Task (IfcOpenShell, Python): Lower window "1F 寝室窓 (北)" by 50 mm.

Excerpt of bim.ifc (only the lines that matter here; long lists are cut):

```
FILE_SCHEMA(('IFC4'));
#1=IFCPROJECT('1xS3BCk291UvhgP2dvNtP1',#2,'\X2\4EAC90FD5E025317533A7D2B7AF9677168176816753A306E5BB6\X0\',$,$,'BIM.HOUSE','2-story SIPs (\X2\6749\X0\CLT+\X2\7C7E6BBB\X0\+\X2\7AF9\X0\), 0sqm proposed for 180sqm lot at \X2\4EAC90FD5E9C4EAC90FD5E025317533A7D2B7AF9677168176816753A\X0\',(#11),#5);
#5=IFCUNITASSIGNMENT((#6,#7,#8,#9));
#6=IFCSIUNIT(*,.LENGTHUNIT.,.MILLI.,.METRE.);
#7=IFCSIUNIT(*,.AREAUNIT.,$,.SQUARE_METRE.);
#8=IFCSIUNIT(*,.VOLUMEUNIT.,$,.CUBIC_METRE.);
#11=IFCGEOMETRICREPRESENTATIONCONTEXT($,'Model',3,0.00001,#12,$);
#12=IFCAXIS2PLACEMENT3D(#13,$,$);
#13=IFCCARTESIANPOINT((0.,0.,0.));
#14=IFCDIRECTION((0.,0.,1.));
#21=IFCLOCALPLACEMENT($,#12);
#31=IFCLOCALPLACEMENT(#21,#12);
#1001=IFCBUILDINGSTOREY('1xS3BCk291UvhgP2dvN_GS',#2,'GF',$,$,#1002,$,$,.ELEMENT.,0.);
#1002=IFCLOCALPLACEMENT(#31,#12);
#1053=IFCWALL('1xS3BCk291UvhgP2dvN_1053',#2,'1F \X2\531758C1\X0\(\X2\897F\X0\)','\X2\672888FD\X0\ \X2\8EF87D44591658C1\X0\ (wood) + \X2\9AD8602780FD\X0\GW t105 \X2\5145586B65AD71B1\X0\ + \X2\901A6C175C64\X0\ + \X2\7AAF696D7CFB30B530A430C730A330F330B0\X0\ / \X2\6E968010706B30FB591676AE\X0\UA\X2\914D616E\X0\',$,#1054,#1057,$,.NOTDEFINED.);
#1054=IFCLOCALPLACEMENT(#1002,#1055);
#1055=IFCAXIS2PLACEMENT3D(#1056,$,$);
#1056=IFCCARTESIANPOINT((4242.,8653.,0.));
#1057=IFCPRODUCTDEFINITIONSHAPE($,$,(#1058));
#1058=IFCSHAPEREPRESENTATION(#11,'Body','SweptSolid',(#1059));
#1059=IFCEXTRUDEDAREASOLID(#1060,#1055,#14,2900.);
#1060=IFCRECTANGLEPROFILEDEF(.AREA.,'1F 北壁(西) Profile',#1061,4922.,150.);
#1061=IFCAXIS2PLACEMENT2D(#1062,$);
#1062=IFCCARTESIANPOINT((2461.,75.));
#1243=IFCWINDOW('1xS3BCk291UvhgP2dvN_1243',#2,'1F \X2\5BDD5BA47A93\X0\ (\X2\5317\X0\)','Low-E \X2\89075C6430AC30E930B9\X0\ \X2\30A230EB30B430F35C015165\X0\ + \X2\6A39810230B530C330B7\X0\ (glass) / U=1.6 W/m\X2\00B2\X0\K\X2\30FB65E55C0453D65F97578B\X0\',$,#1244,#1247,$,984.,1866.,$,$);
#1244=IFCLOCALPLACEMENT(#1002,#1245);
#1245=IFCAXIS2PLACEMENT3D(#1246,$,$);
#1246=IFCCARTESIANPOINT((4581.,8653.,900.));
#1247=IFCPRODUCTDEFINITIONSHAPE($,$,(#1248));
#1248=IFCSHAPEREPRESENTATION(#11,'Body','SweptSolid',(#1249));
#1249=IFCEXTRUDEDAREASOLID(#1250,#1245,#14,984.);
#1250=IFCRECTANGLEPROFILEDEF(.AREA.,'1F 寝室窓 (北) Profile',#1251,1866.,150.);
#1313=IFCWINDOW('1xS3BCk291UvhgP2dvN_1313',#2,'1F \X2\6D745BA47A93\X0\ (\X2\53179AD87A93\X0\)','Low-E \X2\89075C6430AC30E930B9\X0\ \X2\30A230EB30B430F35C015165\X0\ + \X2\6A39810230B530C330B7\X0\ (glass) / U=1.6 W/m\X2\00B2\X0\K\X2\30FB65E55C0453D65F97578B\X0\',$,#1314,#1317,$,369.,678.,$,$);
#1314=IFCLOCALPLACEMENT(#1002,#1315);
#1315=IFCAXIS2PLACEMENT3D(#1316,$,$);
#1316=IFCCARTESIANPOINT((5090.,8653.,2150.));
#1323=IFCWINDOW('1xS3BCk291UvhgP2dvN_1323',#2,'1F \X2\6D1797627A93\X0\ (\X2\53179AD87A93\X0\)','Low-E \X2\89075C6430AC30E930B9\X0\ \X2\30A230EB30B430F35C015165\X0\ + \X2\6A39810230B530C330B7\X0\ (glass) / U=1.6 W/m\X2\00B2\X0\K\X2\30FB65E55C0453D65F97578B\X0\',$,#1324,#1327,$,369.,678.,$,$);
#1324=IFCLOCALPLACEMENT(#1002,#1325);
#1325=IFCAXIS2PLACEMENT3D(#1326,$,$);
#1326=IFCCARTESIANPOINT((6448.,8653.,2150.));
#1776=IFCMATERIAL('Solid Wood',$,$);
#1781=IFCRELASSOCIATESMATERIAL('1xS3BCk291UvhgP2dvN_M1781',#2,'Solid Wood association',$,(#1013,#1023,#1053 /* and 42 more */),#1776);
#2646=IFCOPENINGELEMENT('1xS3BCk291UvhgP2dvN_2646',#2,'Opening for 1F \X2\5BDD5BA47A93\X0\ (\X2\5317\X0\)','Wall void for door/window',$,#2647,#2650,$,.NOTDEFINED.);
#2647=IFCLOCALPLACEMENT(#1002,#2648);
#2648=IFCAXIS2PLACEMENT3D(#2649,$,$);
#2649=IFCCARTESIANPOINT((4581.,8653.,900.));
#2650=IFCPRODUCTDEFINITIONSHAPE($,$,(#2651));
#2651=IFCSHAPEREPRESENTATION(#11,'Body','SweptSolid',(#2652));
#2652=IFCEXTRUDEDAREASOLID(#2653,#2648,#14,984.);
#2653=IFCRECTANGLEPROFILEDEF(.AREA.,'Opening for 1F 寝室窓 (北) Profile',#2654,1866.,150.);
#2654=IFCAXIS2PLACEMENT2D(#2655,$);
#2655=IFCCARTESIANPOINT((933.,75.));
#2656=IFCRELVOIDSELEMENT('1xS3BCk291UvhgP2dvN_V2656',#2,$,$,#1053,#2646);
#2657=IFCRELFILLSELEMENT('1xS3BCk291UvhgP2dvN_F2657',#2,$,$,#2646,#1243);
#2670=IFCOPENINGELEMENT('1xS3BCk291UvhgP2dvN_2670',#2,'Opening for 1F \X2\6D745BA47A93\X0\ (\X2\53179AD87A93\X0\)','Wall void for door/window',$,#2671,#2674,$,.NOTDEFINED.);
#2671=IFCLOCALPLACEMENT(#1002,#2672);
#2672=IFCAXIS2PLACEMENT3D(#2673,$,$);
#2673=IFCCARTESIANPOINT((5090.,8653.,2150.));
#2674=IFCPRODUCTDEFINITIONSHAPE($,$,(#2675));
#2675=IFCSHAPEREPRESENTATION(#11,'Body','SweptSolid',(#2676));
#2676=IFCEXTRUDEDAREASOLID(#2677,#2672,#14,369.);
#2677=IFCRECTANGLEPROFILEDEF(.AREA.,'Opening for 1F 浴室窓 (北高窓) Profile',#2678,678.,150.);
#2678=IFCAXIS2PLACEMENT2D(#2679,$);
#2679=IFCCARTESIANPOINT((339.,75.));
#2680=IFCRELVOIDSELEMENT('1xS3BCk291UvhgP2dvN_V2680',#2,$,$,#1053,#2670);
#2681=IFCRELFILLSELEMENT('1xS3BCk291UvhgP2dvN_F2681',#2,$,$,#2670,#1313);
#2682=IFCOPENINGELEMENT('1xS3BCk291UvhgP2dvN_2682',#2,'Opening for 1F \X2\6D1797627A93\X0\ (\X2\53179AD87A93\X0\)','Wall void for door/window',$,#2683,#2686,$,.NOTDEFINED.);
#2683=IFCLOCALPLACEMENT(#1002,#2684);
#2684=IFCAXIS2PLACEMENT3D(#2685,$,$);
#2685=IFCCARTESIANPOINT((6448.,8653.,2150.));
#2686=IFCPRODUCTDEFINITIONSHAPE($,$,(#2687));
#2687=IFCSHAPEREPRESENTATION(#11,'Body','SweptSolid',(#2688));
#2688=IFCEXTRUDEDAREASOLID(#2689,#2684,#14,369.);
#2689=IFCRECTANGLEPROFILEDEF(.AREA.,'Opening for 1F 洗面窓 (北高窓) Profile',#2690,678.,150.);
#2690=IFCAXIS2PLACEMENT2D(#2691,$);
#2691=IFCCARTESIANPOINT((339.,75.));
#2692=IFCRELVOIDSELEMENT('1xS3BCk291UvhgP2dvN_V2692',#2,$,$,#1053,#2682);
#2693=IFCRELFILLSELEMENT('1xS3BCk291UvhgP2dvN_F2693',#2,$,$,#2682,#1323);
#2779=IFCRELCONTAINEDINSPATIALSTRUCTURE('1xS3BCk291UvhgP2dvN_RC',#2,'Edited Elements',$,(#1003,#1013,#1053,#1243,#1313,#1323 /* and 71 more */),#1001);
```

```python
import numpy as np
import ifcopenshell
import ifcopenshell.api.geometry
import ifcopenshell.util.placement
import ifcopenshell.util.unit

model = ifcopenshell.open("bim.ifc")
unit_scale = ifcopenshell.util.unit.calculate_unit_scale(model)

window = model.by_id(1243)
opening = window.FillsVoids[0].RelatingOpeningElement
dz = -0.05 / unit_scale

shift = np.array([0.0, 0.0, dz])
# The window is not placed relative to its opening, so move both.
for product in (opening, window):
    matrix = ifcopenshell.util.placement.get_local_placement(product.ObjectPlacement)
    matrix[:3, 3] += shift
    ifcopenshell.api.geometry.edit_object_placement(model, product=product, matrix=matrix, is_si=False)

print(f"moved by {dz * unit_scale:+.3f} m")

model.write("bim_edited.ifc")
```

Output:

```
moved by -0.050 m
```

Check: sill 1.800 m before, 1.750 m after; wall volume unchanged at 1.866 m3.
